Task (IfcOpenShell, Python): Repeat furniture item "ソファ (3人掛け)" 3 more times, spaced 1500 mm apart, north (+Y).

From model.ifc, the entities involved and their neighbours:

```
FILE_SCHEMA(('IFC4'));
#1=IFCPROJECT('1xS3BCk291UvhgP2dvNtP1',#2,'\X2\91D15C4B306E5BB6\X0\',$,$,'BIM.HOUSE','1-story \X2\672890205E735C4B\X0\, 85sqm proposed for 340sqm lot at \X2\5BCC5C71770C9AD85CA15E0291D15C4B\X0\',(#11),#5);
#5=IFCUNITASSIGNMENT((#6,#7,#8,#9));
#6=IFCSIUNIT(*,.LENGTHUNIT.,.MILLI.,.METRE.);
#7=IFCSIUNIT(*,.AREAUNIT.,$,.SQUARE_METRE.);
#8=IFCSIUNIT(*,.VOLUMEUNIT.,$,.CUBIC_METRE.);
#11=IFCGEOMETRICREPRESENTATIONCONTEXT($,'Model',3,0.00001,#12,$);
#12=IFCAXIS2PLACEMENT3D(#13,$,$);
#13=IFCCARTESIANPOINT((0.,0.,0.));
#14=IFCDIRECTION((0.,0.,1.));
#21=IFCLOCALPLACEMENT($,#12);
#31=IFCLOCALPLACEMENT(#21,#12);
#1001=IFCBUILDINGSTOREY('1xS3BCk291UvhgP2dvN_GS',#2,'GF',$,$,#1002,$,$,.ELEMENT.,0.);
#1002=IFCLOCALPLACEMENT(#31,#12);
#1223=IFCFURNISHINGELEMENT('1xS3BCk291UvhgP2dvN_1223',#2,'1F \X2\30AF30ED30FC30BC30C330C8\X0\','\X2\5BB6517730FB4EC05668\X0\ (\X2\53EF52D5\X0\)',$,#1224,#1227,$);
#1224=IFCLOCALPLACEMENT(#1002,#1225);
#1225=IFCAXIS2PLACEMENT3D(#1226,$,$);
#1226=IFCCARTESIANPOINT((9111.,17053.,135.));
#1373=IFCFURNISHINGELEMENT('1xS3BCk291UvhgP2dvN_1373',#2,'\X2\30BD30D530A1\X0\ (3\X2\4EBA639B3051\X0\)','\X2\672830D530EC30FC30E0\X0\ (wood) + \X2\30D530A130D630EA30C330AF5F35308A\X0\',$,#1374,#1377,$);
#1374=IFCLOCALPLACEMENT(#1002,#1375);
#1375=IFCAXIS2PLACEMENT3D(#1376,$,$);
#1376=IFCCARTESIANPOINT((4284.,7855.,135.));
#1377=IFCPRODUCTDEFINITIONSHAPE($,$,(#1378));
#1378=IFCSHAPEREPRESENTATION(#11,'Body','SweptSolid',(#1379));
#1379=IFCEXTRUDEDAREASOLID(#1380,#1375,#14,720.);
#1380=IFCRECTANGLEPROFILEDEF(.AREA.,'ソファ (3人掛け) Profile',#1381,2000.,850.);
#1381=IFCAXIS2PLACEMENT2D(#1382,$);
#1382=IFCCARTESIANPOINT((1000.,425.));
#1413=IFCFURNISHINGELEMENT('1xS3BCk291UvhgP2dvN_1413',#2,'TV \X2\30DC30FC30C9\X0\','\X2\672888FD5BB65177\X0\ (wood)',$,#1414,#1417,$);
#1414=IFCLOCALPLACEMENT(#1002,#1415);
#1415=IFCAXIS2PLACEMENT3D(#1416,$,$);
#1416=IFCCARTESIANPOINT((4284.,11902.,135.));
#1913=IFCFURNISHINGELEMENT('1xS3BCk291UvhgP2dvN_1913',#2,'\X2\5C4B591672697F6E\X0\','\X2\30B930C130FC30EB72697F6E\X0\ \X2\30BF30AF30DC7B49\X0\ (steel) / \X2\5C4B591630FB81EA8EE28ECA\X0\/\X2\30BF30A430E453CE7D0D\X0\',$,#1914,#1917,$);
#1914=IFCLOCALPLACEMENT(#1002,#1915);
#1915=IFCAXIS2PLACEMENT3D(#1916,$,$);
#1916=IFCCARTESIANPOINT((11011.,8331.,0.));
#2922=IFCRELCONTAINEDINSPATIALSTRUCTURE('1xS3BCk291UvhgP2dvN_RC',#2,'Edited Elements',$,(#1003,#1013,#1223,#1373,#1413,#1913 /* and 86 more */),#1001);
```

```python
import numpy as np
import ifcopenshell
import ifcopenshell.api.geometry
import ifcopenshell.api.root
import ifcopenshell.util.element
import ifcopenshell.util.placement
import ifcopenshell.util.unit

model = ifcopenshell.open("model.ifc")
unit_scale = ifcopenshell.util.unit.calculate_unit_scale(model)


def reuse_history(source, copy):
    """copy_class also copies each property set's owner history, people and application; keep the originals."""
    for rel in copy.IsDefinedBy:
        if rel.is_a("IfcRelDefinesByProperties") and (history := rel.RelatingPropertyDefinition.OwnerHistory):
            rel.RelatingPropertyDefinition.OwnerHistory = source.OwnerHistory
            ifcopenshell.util.element.remove_deep2(model, history)


source = model.by_guid("1xS3BCk291UvhgP2dvN_1373")
base = ifcopenshell.util.placement.get_local_placement(source.ObjectPlacement)
step = np.array([0.0, 1.0, 0.0]) * 1.5 / unit_scale

for i in range(1, 4):
    copy = ifcopenshell.api.root.copy_class(model, product=source)
    copy.Representation = ifcopenshell.util.element.copy_deep(
        model, source.Representation, exclude=["IfcGeometricRepresentationContext", "IfcRepresentationMap"]
    )
    reuse_history(source, copy)
    matrix = base.copy()
    matrix[:3, 3] += i * step
    print("added at", matrix[:3, 3].round(3) + 0.0)
    ifcopenshell.api.geometry.edit_object_placement(model, product=copy, matrix=matrix, is_si=False)

model.write("model_updated.ifc")
```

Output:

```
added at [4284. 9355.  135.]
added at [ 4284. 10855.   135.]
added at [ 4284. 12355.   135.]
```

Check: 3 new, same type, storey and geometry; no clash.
